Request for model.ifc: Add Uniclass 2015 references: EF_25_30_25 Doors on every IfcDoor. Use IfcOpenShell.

First a look at what the model holds.

```python
import ifcopenshell

model = ifcopenshell.open("model.ifc")
print(model.schema)
print("classifications:", [c.Name for c in model.by_type("IfcClassification")])
for ifc_class in ("IfcDoor", "IfcRoof", "IfcStair", "IfcWall", "IfcWindow"):
    print(ifc_class, len(model.by_type(ifc_class)))
```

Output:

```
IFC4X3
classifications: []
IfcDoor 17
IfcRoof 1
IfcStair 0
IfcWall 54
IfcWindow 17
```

```python
import ifcopenshell
import ifcopenshell.api.classification

model = ifcopenshell.open("model.ifc")

system = ifcopenshell.api.classification.add_classification(model, classification="Uniclass 2015")

codes = {
    "IfcDoor": ("EF_25_30_25", "Doors"),
}
for ifc_class, (code, name) in codes.items():
    products = model.by_type(ifc_class)
    ifcopenshell.api.classification.add_reference(
        model, products=products, classification=system, identification=code, name=name
    )
    print(code, len(products))

model.write("model_updated.ifc")
```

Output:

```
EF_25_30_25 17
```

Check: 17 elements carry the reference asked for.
